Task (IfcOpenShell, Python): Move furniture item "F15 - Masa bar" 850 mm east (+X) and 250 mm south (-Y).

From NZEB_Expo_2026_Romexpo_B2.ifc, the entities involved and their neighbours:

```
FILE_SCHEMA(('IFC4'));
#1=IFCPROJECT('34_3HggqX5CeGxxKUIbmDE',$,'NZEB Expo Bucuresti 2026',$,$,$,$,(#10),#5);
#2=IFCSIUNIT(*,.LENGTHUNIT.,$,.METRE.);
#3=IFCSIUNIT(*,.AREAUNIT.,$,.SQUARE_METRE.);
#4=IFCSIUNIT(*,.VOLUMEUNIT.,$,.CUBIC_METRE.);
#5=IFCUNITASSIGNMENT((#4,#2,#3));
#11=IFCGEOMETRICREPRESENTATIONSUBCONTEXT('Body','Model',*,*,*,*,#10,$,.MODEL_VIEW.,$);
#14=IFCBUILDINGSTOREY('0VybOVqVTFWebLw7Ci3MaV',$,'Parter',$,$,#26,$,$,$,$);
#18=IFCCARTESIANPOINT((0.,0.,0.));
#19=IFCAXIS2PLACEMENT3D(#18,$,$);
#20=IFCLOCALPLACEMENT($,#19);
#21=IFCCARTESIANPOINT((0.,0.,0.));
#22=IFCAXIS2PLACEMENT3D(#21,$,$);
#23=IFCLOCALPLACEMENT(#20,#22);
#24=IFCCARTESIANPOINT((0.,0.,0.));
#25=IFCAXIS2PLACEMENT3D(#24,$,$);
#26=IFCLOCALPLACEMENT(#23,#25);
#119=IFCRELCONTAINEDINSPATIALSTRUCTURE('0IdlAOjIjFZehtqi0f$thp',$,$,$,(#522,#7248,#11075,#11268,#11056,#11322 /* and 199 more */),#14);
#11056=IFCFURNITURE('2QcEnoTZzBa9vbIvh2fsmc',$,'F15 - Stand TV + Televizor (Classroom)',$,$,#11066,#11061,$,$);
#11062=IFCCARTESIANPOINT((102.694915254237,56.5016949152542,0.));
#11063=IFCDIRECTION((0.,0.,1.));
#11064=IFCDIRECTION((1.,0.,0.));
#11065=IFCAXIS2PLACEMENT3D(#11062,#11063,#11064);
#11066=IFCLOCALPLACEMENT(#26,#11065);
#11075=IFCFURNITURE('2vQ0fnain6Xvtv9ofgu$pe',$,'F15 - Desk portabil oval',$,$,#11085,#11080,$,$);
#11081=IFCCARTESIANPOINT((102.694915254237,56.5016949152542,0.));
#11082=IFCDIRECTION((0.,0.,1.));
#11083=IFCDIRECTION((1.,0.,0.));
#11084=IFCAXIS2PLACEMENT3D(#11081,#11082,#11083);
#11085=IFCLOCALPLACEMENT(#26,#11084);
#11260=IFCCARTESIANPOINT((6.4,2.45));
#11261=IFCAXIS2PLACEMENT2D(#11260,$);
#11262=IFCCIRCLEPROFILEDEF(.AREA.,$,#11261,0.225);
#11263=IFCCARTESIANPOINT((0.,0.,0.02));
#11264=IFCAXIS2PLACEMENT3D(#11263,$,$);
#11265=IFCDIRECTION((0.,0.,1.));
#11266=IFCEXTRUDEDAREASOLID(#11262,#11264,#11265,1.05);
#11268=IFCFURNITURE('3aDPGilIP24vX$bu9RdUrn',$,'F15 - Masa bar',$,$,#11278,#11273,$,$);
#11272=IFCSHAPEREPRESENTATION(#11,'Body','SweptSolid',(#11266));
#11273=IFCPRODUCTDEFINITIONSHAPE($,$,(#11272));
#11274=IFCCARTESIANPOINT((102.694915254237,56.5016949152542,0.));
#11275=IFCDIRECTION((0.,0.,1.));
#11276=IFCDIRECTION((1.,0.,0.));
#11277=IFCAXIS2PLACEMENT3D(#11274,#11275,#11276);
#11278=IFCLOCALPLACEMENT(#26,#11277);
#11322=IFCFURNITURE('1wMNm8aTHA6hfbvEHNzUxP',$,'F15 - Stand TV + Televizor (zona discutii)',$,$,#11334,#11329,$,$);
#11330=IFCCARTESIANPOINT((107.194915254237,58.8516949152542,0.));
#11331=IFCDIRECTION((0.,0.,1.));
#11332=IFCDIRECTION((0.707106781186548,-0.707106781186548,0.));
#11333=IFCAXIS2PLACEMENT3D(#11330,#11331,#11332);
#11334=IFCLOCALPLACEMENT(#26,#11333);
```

```python
import ifcopenshell
import ifcopenshell.api.geometry
import ifcopenshell.util.placement
import ifcopenshell.util.unit

model = ifcopenshell.open("NZEB_Expo_2026_Romexpo_B2.ifc")
unit_scale = ifcopenshell.util.unit.calculate_unit_scale(model)

item = model.by_guid("3aDPGilIP24vX$bu9RdUrn")
matrix = ifcopenshell.util.placement.get_local_placement(item.ObjectPlacement)
matrix[0, 3] += 0.85 / unit_scale
matrix[1, 3] -= 0.25 / unit_scale
ifcopenshell.api.geometry.edit_object_placement(model, product=item, matrix=matrix, is_si=False)

print(ifcopenshell.util.placement.get_local_placement(item.ObjectPlacement).round(3) + 0.0)

model.write("NZEB_Expo_2026_Romexpo_B2_edited.ifc")
```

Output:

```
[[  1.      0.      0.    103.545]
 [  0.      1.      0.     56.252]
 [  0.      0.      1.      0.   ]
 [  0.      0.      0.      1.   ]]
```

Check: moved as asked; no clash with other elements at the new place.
